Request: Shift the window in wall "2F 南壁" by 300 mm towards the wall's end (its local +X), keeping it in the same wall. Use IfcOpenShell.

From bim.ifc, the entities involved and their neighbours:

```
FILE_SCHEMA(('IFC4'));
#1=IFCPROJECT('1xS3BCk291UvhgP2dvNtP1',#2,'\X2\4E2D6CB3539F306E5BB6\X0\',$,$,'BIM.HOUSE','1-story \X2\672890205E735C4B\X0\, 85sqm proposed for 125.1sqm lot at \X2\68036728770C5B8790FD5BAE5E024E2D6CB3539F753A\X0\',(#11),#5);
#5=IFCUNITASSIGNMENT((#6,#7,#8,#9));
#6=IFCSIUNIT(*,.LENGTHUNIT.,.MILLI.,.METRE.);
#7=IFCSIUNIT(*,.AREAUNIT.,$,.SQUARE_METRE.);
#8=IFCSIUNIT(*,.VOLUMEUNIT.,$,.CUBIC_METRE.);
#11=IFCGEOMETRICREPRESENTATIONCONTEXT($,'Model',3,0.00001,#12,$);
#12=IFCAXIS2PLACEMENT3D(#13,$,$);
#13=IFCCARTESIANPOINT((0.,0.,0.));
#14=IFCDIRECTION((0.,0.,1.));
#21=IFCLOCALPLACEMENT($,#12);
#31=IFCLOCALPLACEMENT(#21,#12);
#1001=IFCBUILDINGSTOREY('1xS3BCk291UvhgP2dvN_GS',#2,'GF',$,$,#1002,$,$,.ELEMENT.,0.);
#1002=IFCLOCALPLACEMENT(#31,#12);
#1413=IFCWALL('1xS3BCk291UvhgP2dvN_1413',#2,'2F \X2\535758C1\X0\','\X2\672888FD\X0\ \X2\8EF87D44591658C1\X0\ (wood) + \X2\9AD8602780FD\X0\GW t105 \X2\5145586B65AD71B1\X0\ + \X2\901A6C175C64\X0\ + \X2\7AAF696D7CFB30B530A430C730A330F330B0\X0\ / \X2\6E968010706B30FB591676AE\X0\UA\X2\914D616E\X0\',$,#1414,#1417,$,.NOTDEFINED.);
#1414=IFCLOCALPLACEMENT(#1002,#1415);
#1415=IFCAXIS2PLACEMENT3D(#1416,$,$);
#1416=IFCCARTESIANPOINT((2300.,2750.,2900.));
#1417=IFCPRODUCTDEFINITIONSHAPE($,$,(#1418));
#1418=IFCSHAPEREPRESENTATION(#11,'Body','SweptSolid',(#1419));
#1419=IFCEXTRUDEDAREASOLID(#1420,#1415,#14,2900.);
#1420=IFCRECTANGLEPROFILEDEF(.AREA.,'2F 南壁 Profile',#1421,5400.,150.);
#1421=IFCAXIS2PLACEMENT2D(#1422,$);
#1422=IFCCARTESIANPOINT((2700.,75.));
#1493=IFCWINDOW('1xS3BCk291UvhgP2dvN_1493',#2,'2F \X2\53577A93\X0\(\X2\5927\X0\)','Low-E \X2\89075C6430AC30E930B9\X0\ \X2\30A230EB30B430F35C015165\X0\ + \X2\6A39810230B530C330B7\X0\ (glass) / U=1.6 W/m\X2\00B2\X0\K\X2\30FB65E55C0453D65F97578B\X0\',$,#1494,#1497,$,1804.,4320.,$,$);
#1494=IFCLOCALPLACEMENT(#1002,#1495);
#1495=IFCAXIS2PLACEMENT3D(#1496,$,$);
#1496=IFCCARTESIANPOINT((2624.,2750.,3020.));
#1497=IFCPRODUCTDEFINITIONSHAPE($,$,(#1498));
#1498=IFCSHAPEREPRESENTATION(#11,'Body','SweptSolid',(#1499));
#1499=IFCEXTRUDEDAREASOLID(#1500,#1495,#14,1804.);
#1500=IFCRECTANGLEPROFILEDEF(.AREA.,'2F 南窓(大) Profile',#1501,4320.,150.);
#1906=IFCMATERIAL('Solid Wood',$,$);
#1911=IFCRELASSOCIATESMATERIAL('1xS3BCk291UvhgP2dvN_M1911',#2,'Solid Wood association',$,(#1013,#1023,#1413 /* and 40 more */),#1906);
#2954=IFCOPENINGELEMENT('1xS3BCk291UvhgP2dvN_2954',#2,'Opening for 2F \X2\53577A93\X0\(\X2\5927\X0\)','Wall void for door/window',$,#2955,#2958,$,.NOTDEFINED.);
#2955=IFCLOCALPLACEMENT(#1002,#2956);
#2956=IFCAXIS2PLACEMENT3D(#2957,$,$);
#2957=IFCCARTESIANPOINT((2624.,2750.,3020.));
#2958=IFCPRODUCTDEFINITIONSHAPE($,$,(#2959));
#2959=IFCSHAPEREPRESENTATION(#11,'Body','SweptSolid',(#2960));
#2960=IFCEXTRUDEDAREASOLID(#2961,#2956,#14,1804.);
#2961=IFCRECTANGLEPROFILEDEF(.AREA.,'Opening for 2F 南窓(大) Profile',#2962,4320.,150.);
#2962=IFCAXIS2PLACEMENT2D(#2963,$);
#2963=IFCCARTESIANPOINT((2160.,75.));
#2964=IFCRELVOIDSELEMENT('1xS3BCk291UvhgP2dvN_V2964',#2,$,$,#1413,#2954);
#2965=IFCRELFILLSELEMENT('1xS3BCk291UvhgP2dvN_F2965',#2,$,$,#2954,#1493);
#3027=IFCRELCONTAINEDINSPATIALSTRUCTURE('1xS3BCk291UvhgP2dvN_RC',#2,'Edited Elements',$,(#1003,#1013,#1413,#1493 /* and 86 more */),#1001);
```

```python
import ifcopenshell
import ifcopenshell.api.geometry
import ifcopenshell.util.placement

model = ifcopenshell.open("bim.ifc")

window = model.by_guid("1xS3BCk291UvhgP2dvN_1493")
opening = window.FillsVoids[0].RelatingOpeningElement
wall = opening.VoidsElements[0].RelatingBuildingElement

wall_matrix = ifcopenshell.util.placement.get_local_placement(wall.ObjectPlacement)
shift = wall_matrix[:3, 0] * 300.0
before = ifcopenshell.util.placement.get_local_placement(window.ObjectPlacement)[:3, 3].copy()

# The window is not placed relative to its opening, so move both.
for product in (opening, window):
    matrix = ifcopenshell.util.placement.get_local_placement(product.ObjectPlacement)
    matrix[:3, 3] += shift
    ifcopenshell.api.geometry.edit_object_placement(model, product=product, matrix=matrix, is_si=False)

after = ifcopenshell.util.placement.get_local_placement(window.ObjectPlacement)[:3, 3]
print("window moved by", (after - before).round(3) + 0.0)

model.write("bim_updated.ifc")
```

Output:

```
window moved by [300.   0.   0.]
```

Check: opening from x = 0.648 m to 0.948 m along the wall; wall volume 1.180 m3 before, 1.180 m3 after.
